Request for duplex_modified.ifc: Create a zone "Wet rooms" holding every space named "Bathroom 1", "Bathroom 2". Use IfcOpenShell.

First a look at what the model holds.

```python
import ifcopenshell

model = ifcopenshell.open("duplex_modified.ifc")
print(model.schema)
seen = {}
for space in model.by_type("IfcSpace"):
    seen[space.LongName] = seen.get(space.LongName, 0) + 1
for name, count in sorted(seen.items(), key=str):
    print(count, "x", name)
print("zones:", [z.Name for z in model.by_type("IfcZone")][:20])
```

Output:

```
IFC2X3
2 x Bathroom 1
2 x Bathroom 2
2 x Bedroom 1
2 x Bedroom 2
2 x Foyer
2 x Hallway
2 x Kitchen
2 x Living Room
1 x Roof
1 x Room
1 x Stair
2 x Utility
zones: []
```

```python
import ifcopenshell
import ifcopenshell.api.group
import ifcopenshell.api.root

model = ifcopenshell.open("duplex_modified.ifc")

names = {"Bathroom 1", "Bathroom 2"}
spaces = [s for s in model.by_type("IfcSpace") if s.LongName in names]

zone = ifcopenshell.api.root.create_entity(model, ifc_class="IfcZone", name="Wet rooms")
ifcopenshell.api.group.assign_group(model, products=spaces, group=zone)
print(len(spaces), "spaces in", zone.Name)

model.write("duplex_modified_rev.ifc")
```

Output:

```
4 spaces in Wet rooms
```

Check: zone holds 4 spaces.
